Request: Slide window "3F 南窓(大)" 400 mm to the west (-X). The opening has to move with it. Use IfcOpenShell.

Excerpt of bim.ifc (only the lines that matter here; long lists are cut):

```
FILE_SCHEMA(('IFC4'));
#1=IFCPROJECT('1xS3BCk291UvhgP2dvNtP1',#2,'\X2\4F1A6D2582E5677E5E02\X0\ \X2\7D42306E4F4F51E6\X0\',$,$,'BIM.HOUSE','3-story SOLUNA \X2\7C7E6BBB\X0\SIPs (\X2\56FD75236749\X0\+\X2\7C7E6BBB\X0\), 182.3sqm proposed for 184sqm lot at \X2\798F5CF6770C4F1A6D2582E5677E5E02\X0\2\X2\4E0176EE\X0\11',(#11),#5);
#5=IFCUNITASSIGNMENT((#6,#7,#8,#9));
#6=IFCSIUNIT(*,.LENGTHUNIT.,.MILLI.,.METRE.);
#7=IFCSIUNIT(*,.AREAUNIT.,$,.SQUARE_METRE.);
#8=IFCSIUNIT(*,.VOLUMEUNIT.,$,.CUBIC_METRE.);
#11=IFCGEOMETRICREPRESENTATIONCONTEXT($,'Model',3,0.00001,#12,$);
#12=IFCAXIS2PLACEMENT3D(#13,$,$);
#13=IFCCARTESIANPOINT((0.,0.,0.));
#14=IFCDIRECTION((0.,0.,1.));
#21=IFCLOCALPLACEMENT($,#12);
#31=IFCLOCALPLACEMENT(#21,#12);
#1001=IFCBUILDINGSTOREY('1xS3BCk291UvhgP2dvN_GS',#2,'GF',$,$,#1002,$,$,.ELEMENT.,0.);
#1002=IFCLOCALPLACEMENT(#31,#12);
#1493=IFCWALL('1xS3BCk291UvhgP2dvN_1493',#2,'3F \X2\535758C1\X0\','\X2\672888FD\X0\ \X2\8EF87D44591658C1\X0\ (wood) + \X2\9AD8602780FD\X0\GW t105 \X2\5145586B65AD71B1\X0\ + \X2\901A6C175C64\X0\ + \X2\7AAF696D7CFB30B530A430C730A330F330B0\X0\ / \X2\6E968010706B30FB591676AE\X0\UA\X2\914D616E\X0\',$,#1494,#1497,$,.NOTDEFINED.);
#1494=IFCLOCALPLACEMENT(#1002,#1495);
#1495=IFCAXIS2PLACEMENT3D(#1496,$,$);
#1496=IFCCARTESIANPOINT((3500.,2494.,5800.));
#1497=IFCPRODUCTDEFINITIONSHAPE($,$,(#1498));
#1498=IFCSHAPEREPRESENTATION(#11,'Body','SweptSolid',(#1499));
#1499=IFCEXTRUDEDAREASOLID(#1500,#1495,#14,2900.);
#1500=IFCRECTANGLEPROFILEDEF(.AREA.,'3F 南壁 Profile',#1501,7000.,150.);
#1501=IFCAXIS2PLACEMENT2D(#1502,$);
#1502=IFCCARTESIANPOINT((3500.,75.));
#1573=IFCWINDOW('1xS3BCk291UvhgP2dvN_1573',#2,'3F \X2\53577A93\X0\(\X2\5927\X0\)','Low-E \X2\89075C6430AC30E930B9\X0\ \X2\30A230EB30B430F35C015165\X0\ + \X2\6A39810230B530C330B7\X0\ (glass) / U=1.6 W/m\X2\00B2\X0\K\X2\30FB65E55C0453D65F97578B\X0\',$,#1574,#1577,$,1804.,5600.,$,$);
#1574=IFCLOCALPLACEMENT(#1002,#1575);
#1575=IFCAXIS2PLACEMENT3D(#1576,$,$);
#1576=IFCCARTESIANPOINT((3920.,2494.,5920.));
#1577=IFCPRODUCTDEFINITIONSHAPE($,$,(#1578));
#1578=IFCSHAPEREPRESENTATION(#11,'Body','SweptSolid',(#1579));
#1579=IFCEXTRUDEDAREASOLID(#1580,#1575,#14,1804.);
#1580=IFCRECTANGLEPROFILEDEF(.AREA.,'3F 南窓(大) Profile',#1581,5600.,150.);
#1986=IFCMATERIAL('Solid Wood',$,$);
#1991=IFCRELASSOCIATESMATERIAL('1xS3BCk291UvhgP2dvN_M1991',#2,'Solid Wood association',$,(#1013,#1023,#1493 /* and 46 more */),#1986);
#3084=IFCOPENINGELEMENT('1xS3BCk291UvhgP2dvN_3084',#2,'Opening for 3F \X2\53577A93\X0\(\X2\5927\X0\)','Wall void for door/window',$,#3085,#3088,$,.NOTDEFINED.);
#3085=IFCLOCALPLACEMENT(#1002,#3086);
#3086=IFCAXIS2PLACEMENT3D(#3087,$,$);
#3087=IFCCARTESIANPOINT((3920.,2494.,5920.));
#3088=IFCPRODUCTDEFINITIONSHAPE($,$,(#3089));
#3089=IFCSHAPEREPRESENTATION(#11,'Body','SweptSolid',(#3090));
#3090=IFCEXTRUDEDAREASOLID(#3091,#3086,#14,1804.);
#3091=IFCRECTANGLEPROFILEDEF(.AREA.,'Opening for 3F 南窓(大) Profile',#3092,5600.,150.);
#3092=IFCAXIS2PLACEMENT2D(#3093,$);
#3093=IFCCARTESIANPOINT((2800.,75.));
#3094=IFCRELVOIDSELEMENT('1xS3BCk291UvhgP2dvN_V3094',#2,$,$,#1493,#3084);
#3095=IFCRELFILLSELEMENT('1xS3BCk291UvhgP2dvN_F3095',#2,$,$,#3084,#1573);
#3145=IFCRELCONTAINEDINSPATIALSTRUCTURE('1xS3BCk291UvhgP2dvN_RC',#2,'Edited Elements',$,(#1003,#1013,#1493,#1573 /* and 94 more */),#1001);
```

```python
import ifcopenshell
import ifcopenshell.api.geometry
import ifcopenshell.util.placement

model = ifcopenshell.open("bim.ifc")

window = model.by_guid("1xS3BCk291UvhgP2dvN_1573")
opening = window.FillsVoids[0].RelatingOpeningElement
wall = opening.VoidsElements[0].RelatingBuildingElement

wall_matrix = ifcopenshell.util.placement.get_local_placement(wall.ObjectPlacement)
shift = wall_matrix[:3, 0] * -400.0
before = ifcopenshell.util.placement.get_local_placement(window.ObjectPlacement)[:3, 3].copy()

# The window is not placed relative to its opening, so move both.
for product in (opening, window):
    matrix = ifcopenshell.util.placement.get_local_placement(product.ObjectPlacement)
    matrix[:3, 3] += shift
    ifcopenshell.api.geometry.edit_object_placement(model, product=product, matrix=matrix, is_si=False)

after = ifcopenshell.util.placement.get_local_placement(window.ObjectPlacement)[:3, 3]
print("window moved by", (after - before).round(3) + 0.0)

model.write("bim_rev.ifc")
```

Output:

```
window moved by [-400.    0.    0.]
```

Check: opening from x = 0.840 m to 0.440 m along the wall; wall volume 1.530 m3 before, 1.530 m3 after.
